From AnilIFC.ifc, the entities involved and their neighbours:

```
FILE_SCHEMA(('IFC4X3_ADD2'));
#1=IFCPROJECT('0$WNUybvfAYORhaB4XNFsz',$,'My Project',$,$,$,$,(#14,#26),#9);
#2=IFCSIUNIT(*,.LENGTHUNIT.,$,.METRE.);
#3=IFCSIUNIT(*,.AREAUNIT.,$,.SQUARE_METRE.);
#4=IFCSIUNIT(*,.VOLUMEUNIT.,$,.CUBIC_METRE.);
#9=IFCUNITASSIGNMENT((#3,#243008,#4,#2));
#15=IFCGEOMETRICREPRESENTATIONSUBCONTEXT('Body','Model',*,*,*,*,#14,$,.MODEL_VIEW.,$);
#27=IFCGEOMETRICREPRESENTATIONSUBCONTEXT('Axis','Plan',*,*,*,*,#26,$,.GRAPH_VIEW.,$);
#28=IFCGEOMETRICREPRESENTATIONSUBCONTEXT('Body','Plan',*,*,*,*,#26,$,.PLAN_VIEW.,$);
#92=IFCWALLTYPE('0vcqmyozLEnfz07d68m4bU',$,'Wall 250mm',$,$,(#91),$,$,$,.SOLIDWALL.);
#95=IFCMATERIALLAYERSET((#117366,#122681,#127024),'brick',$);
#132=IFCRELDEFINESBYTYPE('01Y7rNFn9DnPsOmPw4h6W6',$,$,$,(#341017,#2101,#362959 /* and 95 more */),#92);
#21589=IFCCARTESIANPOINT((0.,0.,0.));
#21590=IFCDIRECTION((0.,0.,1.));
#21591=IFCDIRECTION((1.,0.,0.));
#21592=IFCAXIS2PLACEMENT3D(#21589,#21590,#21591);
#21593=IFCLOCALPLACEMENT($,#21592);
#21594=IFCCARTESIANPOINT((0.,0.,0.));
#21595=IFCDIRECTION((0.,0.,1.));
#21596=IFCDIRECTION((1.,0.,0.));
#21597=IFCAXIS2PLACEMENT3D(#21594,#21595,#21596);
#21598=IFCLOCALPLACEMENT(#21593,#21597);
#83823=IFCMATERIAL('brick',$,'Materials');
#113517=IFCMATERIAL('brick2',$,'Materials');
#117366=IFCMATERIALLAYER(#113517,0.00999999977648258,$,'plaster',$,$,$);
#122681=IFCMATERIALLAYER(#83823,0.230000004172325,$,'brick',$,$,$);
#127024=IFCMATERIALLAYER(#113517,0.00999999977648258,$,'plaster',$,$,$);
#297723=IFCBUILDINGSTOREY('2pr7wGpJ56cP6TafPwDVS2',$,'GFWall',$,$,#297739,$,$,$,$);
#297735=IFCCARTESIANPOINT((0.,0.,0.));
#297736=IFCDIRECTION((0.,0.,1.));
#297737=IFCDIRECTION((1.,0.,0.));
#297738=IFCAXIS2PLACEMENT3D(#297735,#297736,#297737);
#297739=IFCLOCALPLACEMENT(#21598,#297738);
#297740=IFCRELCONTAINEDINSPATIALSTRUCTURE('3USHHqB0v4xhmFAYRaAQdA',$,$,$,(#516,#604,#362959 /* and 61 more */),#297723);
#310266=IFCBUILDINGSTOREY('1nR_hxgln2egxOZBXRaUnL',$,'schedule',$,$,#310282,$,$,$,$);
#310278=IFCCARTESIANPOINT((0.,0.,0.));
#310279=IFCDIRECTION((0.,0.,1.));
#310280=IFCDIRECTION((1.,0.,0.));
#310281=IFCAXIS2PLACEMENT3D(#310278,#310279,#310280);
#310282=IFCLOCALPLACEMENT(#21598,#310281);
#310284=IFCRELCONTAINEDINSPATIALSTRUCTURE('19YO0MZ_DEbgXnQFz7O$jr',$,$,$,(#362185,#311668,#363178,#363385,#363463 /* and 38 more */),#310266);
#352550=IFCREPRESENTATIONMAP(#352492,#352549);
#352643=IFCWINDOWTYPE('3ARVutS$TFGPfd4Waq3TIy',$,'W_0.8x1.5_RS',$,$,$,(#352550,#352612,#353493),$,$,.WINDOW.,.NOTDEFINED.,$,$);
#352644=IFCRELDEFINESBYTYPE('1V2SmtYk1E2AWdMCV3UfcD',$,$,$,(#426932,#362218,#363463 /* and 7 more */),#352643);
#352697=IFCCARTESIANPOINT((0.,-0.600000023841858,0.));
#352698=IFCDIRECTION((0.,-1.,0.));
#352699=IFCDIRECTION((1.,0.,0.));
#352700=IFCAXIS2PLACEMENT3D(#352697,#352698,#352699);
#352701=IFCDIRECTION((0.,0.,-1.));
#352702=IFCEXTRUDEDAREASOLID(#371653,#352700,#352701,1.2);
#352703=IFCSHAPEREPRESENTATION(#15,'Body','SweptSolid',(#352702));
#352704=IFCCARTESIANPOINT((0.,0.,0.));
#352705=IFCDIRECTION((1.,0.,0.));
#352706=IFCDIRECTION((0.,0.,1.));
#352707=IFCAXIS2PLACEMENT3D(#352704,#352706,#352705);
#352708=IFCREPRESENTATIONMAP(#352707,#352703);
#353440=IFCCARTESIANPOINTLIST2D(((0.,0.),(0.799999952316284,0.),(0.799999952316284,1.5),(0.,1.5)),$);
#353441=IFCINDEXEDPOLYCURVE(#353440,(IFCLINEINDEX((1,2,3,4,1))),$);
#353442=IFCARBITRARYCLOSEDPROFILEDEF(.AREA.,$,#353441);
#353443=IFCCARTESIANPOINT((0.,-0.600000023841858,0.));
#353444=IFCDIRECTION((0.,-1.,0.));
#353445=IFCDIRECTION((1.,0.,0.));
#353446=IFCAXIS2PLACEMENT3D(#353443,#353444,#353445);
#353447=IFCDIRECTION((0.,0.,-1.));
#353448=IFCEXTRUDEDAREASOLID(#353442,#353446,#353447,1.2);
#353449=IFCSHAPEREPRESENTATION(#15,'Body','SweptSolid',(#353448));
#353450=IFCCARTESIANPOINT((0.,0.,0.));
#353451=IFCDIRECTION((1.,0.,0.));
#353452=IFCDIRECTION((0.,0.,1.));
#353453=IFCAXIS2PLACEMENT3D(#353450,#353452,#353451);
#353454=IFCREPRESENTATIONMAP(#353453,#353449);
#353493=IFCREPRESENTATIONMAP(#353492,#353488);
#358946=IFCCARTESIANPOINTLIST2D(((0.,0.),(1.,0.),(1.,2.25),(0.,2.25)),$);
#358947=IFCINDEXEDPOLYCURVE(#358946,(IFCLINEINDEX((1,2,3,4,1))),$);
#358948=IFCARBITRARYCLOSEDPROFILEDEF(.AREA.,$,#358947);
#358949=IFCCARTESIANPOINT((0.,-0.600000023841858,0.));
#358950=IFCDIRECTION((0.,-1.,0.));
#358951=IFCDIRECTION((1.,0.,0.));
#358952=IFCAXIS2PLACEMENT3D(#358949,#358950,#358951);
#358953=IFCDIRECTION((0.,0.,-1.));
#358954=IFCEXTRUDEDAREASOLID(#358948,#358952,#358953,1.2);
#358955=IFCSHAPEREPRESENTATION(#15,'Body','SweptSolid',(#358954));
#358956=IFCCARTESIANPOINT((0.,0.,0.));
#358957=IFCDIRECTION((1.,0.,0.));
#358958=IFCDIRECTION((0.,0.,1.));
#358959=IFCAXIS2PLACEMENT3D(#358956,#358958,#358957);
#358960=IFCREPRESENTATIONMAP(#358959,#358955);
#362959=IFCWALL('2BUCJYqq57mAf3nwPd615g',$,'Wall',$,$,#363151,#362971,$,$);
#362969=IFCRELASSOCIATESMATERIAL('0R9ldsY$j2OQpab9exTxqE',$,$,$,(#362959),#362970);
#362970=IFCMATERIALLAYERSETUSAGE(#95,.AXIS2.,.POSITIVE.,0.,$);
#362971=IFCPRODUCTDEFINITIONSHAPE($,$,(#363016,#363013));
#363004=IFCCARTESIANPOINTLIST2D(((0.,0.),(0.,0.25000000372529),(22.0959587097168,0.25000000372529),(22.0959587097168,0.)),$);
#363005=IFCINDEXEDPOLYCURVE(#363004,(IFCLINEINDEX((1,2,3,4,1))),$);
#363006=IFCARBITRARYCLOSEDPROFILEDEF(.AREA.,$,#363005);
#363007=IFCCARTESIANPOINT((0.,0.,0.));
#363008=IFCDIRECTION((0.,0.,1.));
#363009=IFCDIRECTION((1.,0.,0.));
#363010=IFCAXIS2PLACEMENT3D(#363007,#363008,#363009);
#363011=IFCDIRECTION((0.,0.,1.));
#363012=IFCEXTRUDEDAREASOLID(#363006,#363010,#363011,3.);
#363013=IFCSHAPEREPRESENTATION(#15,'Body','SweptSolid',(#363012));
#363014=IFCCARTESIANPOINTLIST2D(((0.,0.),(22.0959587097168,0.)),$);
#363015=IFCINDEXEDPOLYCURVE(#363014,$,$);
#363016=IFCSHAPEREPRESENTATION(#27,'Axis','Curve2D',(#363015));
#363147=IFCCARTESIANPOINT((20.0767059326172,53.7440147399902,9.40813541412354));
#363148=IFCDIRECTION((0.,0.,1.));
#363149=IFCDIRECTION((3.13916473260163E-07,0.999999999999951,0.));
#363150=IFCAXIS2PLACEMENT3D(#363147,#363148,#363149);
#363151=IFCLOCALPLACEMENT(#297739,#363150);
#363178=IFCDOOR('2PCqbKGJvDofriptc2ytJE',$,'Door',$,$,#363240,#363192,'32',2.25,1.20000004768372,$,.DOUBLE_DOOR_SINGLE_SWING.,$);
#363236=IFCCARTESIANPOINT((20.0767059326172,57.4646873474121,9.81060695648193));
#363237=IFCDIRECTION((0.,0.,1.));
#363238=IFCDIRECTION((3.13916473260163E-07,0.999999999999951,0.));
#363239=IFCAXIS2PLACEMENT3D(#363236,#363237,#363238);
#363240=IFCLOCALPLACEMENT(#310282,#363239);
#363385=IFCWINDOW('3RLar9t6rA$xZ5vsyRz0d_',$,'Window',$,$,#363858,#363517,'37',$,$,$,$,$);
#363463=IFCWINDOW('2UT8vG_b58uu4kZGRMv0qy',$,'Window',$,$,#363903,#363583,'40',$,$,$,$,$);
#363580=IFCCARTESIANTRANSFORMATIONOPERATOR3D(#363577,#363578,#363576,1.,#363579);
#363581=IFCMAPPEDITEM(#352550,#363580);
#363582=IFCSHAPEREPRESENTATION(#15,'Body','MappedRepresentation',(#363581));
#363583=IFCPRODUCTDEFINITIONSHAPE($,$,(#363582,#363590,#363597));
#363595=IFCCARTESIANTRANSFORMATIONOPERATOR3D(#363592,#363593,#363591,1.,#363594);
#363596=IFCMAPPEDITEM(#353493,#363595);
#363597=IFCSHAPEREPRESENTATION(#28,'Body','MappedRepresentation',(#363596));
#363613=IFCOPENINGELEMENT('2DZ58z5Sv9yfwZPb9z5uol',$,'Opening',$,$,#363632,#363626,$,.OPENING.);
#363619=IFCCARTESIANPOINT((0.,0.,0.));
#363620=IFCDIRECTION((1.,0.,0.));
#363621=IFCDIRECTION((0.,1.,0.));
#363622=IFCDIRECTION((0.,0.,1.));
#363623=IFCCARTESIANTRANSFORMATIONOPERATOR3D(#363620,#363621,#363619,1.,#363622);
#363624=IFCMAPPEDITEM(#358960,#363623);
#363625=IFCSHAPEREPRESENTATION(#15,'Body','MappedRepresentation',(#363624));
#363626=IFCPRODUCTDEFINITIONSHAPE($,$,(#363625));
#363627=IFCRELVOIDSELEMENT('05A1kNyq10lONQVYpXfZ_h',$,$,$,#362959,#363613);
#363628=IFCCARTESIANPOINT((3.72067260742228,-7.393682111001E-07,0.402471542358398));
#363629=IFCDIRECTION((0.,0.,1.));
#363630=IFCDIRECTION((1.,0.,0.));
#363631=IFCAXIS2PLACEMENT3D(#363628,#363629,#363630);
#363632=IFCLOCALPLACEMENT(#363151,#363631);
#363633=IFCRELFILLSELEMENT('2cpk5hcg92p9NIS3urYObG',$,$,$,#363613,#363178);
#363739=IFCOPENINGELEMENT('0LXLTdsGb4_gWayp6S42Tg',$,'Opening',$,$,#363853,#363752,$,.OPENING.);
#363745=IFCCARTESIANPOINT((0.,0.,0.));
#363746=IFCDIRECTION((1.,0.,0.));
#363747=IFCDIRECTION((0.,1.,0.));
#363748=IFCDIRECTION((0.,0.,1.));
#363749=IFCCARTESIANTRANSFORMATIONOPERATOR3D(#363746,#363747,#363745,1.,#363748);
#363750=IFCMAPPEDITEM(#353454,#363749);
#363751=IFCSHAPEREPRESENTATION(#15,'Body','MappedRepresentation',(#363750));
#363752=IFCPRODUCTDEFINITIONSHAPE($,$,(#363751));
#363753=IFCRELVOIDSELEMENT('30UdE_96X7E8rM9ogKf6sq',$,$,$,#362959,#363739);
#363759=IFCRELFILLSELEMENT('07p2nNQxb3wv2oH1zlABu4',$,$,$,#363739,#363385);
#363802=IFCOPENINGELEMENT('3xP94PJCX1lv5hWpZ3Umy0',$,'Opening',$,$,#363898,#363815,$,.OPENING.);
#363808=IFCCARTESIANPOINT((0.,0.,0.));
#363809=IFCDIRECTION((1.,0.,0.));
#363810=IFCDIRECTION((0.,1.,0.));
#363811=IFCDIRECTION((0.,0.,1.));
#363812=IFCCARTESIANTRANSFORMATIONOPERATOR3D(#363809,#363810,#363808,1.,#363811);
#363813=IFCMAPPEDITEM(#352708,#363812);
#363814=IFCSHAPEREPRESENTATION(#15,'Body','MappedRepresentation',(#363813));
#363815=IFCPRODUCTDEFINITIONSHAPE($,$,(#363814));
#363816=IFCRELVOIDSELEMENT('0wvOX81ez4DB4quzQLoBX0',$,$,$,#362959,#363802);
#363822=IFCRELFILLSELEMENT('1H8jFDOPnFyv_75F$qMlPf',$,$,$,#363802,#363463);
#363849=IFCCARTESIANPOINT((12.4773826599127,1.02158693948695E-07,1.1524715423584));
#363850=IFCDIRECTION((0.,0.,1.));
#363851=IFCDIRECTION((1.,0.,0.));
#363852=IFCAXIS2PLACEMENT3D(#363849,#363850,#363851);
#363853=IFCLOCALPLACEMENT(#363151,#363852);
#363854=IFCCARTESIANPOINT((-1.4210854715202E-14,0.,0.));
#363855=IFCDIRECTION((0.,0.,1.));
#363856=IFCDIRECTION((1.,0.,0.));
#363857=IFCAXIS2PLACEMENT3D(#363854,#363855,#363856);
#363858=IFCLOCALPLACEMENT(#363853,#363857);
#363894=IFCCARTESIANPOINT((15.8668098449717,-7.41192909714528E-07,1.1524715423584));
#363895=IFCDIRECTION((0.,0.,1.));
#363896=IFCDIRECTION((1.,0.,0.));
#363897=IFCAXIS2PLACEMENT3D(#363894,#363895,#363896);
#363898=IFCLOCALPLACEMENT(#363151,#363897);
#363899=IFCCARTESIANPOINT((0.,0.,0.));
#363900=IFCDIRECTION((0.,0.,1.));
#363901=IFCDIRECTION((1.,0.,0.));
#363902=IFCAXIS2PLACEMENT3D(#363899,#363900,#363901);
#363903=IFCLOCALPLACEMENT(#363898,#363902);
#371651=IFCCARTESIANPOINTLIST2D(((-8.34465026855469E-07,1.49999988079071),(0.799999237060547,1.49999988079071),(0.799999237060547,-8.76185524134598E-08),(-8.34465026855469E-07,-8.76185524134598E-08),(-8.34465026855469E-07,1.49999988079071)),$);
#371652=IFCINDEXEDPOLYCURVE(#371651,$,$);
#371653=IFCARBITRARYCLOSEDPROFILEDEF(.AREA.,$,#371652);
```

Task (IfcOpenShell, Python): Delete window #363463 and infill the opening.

```python
import ifcopenshell
import ifcopenshell.api.feature
import ifcopenshell.api.root
import ifcopenshell.geom
import ifcopenshell.util.shape

model = ifcopenshell.open("AnilIFC.ifc")
settings = ifcopenshell.geom.settings()


def volume(element):
    """Net volume in cubic metres, openings subtracted."""
    shape = ifcopenshell.geom.create_shape(settings, element)
    return ifcopenshell.util.shape.get_volume(shape.geometry)


window = model.by_guid("2UT8vG_b58uu4kZGRMv0qy")
opening = window.FillsVoids[0].RelatingOpeningElement
wall = opening.VoidsElements[0].RelatingBuildingElement
before = volume(wall)

ifcopenshell.api.root.remove_product(model, product=window)
ifcopenshell.api.feature.remove_feature(model, feature=opening)

after = volume(wall)

print(f"wall volume {before:.3f} -> {after:.3f} m3")

model.write("AnilIFC-out.ifc")
```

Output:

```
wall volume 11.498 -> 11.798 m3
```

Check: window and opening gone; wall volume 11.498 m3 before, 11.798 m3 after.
